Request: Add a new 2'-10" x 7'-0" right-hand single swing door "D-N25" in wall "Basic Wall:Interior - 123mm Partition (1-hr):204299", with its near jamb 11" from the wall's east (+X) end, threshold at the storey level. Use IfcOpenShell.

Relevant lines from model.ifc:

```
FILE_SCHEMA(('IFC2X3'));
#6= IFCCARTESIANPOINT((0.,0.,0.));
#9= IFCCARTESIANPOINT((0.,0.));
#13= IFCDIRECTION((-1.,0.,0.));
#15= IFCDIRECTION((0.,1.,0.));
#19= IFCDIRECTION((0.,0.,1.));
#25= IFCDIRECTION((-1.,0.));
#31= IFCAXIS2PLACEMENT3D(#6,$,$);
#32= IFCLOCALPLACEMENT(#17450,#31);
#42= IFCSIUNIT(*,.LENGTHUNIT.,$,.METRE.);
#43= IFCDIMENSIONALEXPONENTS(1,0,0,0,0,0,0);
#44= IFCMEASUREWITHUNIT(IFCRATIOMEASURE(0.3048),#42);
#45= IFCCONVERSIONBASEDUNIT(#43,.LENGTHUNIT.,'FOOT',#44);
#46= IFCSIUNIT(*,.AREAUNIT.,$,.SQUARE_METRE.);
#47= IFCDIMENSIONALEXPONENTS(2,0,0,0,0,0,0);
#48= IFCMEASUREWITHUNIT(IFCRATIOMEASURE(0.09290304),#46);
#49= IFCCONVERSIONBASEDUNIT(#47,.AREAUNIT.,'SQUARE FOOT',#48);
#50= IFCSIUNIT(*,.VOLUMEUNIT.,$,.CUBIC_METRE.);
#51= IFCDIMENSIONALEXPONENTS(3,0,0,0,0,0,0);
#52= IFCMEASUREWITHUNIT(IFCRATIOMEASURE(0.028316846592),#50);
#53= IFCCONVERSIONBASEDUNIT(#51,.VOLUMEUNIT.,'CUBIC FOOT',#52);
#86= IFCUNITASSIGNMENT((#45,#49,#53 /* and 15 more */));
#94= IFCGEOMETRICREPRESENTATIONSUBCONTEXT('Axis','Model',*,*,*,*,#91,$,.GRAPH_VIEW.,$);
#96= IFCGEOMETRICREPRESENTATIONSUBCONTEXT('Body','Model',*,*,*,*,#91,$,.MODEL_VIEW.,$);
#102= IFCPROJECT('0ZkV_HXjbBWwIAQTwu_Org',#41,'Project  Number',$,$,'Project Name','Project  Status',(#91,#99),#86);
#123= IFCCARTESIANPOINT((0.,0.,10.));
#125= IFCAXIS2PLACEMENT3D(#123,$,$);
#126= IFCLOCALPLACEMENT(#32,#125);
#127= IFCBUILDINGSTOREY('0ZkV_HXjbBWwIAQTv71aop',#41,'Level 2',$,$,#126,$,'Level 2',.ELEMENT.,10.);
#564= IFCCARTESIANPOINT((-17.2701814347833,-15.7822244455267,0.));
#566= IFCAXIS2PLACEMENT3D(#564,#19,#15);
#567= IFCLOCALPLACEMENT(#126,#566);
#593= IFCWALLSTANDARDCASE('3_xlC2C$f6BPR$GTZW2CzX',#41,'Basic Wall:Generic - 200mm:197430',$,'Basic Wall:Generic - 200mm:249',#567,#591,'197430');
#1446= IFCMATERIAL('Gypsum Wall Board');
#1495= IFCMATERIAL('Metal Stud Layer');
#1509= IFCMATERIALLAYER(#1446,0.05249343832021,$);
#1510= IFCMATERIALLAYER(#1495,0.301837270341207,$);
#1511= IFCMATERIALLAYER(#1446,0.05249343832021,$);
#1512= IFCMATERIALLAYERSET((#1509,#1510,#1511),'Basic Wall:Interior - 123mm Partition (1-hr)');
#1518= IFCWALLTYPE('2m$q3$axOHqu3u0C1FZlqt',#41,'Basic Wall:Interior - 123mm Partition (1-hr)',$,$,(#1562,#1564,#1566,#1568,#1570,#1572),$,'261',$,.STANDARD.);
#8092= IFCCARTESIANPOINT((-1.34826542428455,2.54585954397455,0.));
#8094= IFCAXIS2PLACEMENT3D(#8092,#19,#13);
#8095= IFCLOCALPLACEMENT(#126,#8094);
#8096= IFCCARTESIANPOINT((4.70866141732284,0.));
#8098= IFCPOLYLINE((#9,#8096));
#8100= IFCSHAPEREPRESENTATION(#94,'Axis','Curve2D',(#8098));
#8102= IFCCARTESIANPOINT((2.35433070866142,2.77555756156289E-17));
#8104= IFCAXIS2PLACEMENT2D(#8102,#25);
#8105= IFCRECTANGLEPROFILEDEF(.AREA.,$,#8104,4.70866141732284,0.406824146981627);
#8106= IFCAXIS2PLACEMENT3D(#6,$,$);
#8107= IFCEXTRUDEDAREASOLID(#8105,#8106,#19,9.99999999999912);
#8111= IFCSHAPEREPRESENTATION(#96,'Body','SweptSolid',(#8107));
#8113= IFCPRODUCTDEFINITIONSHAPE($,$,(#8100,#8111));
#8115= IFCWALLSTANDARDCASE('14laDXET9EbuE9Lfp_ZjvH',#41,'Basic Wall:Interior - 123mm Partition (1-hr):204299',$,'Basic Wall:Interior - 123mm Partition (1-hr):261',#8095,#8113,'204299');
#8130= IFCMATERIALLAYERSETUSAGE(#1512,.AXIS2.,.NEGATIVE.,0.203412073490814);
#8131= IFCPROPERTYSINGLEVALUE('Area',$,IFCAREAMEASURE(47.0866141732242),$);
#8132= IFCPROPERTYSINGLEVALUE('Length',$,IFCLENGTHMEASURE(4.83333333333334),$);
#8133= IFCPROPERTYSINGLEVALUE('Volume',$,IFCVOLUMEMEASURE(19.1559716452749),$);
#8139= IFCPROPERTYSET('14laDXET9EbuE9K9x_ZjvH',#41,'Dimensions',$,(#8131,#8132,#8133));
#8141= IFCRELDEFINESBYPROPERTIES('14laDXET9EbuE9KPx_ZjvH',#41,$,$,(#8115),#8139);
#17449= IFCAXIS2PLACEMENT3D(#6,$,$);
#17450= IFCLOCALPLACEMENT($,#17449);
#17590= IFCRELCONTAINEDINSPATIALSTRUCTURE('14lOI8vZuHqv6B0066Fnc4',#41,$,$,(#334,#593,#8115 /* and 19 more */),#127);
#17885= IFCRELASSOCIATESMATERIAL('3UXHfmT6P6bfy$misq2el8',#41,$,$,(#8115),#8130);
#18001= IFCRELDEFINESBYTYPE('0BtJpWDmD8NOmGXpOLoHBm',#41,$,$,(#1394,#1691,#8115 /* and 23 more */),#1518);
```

```python
import numpy as np
import ifcopenshell
import ifcopenshell.api.feature
import ifcopenshell.api.geometry
import ifcopenshell.api.pset
import ifcopenshell.api.root
import ifcopenshell.api.spatial
import ifcopenshell.api.type
import ifcopenshell.geom
import ifcopenshell.util.element
import ifcopenshell.util.placement
import ifcopenshell.util.representation
import ifcopenshell.util.shape
import ifcopenshell.util.unit

model = ifcopenshell.open("model.ifc")
unit_scale = ifcopenshell.util.unit.calculate_unit_scale(model)
area_scale = ifcopenshell.util.unit.calculate_unit_scale(model, "AREAUNIT")
volume_scale = ifcopenshell.util.unit.calculate_unit_scale(model, "VOLUMEUNIT")
settings = ifcopenshell.geom.settings()


def volume(element):
    """Net volume in cubic metres, openings subtracted."""
    shape = ifcopenshell.geom.create_shape(settings, element)
    return ifcopenshell.util.shape.get_volume(shape.geometry)


wall = model.by_id(8115)
storey = ifcopenshell.util.element.get_container(wall, ifc_class="IfcBuildingStorey")
context = ifcopenshell.util.representation.get_context(model, "Model", "Body", "MODEL_VIEW")
before = volume(wall)

width, height, from_end, sill = 0.8636, 2.1336, 0.2794, 0.0  # metres

# The wall runs along its own X axis, and the end named is its -X end.
wall_shape = ifcopenshell.geom.create_shape(settings, wall)
x, y, z = ifcopenshell.util.shape.get_vertices(wall_shape.geometry).T
start = x.min() + from_end
face, thickness = float(y.min()), float(y.max() - y.min())
wall_matrix = ifcopenshell.util.placement.get_local_placement(wall.ObjectPlacement)
level = ifcopenshell.util.placement.get_local_placement(storey.ObjectPlacement)[2, 3]


def in_wall(x, y):
    """Placement at x, y metres in the wall's axes, at sill height."""
    matrix = wall_matrix.copy()
    matrix[:, 3] = wall_matrix @ np.array([x / unit_scale, y / unit_scale, 0.0, 1.0])
    matrix[2, 3] = level + sill / unit_scale
    return matrix


# Opening: a box that overshoots both wall faces by 50 mm.
opening = ifcopenshell.api.root.create_entity(model, ifc_class="IfcOpeningElement")
box = ifcopenshell.api.geometry.add_wall_representation(
    model, context=context, length=width, height=height, thickness=thickness + 0.1
)
ifcopenshell.api.geometry.assign_representation(model, product=opening, representation=box)
ifcopenshell.api.geometry.edit_object_placement(model, product=opening, matrix=in_wall(start, face - 0.05), is_si=False)
ifcopenshell.api.feature.add_feature(model, feature=opening, element=wall)

door = ifcopenshell.api.root.create_entity(model, ifc_class="IfcDoor", name="D-N25")
door.OverallWidth, door.OverallHeight = width / unit_scale, height / unit_scale
body = ifcopenshell.api.geometry.add_door_representation(
    model,
    context=context,
    overall_width=door.OverallWidth,
    overall_height=door.OverallHeight,
    operation_type="SINGLE_SWING_RIGHT",
    lining_properties={"LiningDepth": thickness / unit_scale, "ThresholdDepth": thickness / unit_scale},
)
ifcopenshell.api.geometry.assign_representation(model, product=door, representation=body)
ifcopenshell.api.spatial.assign_container(model, products=[door], relating_structure=storey)
fills = ifcopenshell.api.feature.add_filling(model, opening=opening, element=door)
fills.OwnerHistory = door.OwnerHistory  # required in IFC2X3

# IFC2X3 keeps the operation on the door style.
style = ifcopenshell.api.root.create_entity(model, ifc_class="IfcDoorStyle", name="D-N25")
style.OperationType, style.ConstructionType = "SINGLE_SWING_RIGHT", "NOTDEFINED"
style.ParameterTakesPrecedence = style.Sizeable = False
ifcopenshell.api.type.assign_type(model, related_objects=[door], relating_type=style)

# The lining spans the wall, so the door starts at the wall face.
ifcopenshell.api.geometry.edit_object_placement(model, product=door, matrix=in_wall(start, face), is_si=False)

after = volume(wall)

# Update the wall's stored quantities.
pset = model.by_id(ifcopenshell.util.element.get_pset(wall, "Dimensions", should_inherit=False)["id"])
ifcopenshell.api.pset.edit_pset(model, pset=pset, properties={
    "Area": model.create_entity("IfcAreaMeasure", after / thickness / area_scale),
    "Volume": model.create_entity("IfcVolumeMeasure", after / volume_scale),
})

print(f"wall volume {before:.3f} -> {after:.3f} m3")

model.write("model_v2.ifc")
```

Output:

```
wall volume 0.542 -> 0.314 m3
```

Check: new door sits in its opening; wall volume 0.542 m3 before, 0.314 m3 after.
